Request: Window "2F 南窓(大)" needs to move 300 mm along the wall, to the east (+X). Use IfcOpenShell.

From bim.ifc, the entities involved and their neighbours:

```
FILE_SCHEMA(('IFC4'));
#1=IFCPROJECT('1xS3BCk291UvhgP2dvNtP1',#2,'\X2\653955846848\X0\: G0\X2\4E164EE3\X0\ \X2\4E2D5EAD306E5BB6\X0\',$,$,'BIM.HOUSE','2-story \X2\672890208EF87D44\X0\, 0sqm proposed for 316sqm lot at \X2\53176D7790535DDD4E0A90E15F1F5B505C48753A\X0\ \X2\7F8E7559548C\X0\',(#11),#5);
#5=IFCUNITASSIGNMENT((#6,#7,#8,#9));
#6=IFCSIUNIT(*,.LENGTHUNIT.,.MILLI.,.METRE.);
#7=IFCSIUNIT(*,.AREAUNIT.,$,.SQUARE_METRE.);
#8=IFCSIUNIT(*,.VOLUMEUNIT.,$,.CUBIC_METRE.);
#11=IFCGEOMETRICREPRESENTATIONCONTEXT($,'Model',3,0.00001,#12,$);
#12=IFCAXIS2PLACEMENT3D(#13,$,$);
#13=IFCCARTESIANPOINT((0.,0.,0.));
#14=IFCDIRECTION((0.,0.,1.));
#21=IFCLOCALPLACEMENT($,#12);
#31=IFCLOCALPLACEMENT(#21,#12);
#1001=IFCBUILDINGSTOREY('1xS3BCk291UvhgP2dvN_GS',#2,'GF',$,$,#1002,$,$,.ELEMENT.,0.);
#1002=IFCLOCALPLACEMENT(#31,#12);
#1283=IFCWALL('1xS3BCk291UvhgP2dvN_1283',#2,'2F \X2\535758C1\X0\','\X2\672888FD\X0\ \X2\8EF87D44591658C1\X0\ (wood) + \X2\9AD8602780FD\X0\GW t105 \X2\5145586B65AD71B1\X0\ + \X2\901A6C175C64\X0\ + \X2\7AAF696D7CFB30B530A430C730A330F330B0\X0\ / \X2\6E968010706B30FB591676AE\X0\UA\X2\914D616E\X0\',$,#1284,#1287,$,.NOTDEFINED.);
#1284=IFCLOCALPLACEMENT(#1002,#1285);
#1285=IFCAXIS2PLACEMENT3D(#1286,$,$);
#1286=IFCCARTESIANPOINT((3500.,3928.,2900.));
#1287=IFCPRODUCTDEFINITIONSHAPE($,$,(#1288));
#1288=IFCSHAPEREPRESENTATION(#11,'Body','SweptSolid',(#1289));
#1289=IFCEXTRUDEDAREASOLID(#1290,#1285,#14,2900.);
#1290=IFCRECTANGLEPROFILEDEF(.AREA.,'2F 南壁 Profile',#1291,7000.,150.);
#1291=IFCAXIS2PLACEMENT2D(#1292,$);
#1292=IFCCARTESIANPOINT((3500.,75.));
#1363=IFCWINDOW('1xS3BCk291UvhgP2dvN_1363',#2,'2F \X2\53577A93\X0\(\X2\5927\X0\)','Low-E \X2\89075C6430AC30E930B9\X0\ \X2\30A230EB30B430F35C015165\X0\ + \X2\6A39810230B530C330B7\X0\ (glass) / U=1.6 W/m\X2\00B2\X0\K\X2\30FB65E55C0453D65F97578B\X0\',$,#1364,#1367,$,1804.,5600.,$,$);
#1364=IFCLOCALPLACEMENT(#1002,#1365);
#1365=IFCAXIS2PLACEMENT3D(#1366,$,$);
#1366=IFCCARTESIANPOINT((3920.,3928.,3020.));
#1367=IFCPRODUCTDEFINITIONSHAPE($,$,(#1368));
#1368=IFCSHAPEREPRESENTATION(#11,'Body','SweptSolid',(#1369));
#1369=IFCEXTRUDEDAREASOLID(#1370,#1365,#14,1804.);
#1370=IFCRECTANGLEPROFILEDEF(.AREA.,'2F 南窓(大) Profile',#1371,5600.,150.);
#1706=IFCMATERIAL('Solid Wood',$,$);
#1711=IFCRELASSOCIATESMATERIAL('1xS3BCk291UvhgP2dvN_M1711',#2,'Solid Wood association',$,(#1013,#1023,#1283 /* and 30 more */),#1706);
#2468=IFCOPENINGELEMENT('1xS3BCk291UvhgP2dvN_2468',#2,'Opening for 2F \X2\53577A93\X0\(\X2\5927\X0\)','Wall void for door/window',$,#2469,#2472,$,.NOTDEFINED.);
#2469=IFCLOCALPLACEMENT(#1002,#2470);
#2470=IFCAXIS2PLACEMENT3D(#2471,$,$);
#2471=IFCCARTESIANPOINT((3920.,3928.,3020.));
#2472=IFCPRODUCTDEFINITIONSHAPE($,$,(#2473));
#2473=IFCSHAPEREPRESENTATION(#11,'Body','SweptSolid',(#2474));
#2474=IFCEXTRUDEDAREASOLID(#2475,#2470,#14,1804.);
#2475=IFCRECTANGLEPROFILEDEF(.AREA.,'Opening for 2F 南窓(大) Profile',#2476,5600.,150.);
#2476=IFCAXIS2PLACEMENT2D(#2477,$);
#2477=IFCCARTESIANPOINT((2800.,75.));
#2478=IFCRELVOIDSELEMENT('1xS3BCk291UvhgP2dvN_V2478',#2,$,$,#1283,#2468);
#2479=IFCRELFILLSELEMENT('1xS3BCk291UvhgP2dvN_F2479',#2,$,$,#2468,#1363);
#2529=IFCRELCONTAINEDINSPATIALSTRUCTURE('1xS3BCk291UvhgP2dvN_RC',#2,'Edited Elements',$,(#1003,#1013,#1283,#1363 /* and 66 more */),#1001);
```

```python
import ifcopenshell
import ifcopenshell.api.geometry
import ifcopenshell.util.placement
import ifcopenshell.util.unit

model = ifcopenshell.open("bim.ifc")
unit_scale = ifcopenshell.util.unit.calculate_unit_scale(model)

window = model.by_id(1363)
opening = window.FillsVoids[0].RelatingOpeningElement
wall = opening.VoidsElements[0].RelatingBuildingElement

wall_matrix = ifcopenshell.util.placement.get_local_placement(wall.ObjectPlacement)
shift = wall_matrix[:3, 0] * 0.3 / unit_scale
before = ifcopenshell.util.placement.get_local_placement(window.ObjectPlacement)[:3, 3].copy()

# The window is not placed relative to its opening, so move both.
for product in (opening, window):
    matrix = ifcopenshell.util.placement.get_local_placement(product.ObjectPlacement)
    matrix[:3, 3] += shift
    ifcopenshell.api.geometry.edit_object_placement(model, product=product, matrix=matrix, is_si=False)

after = ifcopenshell.util.placement.get_local_placement(window.ObjectPlacement)[:3, 3]
print("window moved by", (after - before).round(3) + 0.0)

model.write("bim_v2.ifc")
```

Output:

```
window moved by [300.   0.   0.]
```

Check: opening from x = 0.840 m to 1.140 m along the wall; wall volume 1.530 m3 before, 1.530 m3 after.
